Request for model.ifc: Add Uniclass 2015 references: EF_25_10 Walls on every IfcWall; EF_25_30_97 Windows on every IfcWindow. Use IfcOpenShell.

First a look at what the model holds.

```python
import ifcopenshell

model = ifcopenshell.open("model.ifc")
print(model.schema)
print("classifications:", [c.Name for c in model.by_type("IfcClassification")])
for ifc_class in ("IfcDoor", "IfcRoof", "IfcStair", "IfcWall", "IfcWindow"):
    print(ifc_class, len(model.by_type(ifc_class)))
```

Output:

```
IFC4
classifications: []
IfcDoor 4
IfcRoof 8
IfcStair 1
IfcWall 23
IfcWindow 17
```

```python
import ifcopenshell
import ifcopenshell.api.classification

model = ifcopenshell.open("model.ifc")

system = ifcopenshell.api.classification.add_classification(model, classification="Uniclass 2015")

codes = {
    "IfcWall": ("EF_25_10", "Walls"),
    "IfcWindow": ("EF_25_30_97", "Windows"),
}
for ifc_class, (code, name) in codes.items():
    products = model.by_type(ifc_class)
    ifcopenshell.api.classification.add_reference(
        model, products=products, classification=system, identification=code, name=name
    )
    print(code, len(products))

model.write("model_rev.ifc")
```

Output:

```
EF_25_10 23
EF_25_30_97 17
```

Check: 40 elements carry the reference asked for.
